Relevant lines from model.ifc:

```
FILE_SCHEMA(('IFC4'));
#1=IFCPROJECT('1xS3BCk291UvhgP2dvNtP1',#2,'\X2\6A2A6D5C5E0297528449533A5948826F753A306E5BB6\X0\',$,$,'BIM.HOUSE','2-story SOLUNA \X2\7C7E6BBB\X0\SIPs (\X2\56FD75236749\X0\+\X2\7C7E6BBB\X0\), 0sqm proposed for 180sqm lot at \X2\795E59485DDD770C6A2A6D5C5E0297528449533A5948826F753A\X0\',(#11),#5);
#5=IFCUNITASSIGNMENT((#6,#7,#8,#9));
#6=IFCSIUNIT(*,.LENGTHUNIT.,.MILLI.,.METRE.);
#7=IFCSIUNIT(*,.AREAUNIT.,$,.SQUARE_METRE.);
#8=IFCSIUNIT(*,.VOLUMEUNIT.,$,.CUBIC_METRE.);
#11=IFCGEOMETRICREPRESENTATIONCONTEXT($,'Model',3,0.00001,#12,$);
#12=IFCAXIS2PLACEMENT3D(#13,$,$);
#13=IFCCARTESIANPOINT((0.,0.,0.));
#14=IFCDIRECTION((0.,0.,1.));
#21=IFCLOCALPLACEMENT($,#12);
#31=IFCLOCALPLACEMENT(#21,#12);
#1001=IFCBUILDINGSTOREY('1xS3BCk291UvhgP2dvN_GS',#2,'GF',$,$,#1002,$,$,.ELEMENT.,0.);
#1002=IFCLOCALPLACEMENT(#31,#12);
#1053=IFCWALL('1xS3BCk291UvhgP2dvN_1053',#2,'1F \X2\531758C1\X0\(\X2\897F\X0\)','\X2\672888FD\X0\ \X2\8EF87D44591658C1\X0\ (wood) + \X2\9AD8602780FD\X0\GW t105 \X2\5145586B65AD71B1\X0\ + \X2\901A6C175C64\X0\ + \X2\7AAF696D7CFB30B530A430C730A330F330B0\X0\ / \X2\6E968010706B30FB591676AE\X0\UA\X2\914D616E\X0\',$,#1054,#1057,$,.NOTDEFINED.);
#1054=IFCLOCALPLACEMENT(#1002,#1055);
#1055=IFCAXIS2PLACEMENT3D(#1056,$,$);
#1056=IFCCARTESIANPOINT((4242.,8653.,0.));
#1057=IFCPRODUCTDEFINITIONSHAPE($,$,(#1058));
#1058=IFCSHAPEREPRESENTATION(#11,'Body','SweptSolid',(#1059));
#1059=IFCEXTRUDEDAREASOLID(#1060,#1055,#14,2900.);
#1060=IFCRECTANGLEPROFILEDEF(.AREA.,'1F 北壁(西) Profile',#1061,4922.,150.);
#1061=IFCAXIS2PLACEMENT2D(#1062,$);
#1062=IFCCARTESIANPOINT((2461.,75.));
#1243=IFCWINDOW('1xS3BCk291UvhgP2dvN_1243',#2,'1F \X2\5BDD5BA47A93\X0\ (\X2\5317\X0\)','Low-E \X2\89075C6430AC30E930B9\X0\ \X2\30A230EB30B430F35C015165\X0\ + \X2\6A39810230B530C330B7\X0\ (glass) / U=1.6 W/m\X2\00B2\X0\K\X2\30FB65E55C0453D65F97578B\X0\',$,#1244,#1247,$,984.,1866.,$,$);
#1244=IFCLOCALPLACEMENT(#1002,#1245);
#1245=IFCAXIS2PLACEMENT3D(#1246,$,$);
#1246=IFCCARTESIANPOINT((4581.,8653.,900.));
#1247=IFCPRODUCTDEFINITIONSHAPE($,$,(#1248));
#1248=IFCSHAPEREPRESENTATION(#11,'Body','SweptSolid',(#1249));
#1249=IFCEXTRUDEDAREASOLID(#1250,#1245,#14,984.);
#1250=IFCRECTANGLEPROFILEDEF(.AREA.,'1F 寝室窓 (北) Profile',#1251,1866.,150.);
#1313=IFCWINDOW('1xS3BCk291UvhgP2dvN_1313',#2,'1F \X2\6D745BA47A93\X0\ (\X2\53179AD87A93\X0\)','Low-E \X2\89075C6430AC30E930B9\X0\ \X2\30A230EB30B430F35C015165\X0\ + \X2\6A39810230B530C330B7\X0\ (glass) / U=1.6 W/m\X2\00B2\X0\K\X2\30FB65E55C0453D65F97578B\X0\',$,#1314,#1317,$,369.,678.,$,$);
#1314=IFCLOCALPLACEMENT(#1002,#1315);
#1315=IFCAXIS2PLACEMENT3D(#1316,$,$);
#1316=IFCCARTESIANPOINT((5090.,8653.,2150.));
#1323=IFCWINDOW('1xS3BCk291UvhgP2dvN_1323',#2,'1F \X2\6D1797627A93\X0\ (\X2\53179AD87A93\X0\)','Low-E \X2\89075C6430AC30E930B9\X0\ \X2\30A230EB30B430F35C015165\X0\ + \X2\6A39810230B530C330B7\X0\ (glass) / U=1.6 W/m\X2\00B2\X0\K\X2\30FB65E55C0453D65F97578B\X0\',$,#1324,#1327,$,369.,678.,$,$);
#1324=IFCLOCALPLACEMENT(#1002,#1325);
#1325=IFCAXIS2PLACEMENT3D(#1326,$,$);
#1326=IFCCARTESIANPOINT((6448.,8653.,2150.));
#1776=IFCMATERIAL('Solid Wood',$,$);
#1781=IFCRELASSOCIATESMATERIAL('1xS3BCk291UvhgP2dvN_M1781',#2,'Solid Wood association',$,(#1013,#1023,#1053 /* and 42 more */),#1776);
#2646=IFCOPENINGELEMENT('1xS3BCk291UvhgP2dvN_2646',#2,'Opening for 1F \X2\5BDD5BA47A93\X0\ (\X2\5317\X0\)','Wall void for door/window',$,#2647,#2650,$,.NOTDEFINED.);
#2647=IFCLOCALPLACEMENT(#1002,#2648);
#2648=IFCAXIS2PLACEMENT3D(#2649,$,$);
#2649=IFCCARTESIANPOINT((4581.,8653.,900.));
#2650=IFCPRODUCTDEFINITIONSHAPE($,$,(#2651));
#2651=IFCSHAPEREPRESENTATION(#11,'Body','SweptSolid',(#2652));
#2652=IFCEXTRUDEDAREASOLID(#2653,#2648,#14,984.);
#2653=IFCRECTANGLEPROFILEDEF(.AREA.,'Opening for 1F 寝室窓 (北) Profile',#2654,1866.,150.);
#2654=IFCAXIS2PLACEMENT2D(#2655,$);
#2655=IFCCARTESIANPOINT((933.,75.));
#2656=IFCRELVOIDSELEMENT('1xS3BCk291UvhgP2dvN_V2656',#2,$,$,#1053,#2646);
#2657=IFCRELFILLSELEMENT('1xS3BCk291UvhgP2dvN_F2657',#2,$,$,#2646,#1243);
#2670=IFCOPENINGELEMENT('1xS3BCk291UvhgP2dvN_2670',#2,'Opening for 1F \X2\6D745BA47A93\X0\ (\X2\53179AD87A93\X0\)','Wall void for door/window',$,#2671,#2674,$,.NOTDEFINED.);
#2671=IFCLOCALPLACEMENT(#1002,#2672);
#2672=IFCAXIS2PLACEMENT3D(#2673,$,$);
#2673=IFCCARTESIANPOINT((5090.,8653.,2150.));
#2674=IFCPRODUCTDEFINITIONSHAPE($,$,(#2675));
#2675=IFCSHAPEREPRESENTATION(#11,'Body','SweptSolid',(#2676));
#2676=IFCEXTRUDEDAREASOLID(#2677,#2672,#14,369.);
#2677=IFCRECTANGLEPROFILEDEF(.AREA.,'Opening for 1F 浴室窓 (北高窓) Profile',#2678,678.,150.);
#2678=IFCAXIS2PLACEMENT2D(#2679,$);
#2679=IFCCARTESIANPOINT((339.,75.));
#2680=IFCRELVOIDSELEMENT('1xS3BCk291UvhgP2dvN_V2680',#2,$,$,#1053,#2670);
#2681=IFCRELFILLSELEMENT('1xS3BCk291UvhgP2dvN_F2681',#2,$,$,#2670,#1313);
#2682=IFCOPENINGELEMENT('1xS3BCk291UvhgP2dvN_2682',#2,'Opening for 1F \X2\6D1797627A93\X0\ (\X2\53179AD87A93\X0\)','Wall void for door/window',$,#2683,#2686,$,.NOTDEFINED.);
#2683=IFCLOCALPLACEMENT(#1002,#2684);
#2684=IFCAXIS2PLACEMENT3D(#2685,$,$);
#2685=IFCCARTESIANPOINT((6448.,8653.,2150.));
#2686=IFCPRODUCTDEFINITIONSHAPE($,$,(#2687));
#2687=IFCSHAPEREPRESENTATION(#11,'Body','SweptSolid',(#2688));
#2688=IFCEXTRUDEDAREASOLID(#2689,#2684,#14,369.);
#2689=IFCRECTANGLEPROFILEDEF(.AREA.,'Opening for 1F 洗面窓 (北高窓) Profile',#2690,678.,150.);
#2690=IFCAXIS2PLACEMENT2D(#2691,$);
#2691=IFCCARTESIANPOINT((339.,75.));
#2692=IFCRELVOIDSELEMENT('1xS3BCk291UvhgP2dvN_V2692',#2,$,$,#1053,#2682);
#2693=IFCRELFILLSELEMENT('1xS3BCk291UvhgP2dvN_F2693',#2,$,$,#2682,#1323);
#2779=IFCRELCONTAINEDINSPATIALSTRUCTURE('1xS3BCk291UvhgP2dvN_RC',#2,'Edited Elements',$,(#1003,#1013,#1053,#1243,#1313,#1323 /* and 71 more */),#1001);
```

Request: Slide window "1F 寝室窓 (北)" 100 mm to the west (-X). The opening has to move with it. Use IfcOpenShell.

```python
import ifcopenshell
import ifcopenshell.api.geometry
import ifcopenshell.util.placement
import ifcopenshell.util.unit

model = ifcopenshell.open("model.ifc")
unit_scale = ifcopenshell.util.unit.calculate_unit_scale(model)

window = model.by_guid("1xS3BCk291UvhgP2dvN_1243")
opening = window.FillsVoids[0].RelatingOpeningElement
wall = opening.VoidsElements[0].RelatingBuildingElement

wall_matrix = ifcopenshell.util.placement.get_local_placement(wall.ObjectPlacement)
shift = wall_matrix[:3, 0] * -0.1 / unit_scale
before = ifcopenshell.util.placement.get_local_placement(window.ObjectPlacement)[:3, 3].copy()

# The window is not placed relative to its opening, so move both.
for product in (opening, window):
    matrix = ifcopenshell.util.placement.get_local_placement(product.ObjectPlacement)
    matrix[:3, 3] += shift
    ifcopenshell.api.geometry.edit_object_placement(model, product=product, matrix=matrix, is_si=False)

after = ifcopenshell.util.placement.get_local_placement(window.ObjectPlacement)[:3, 3]
print("window moved by", (after - before).round(3) + 0.0)

model.write("model_rev.ifc")
```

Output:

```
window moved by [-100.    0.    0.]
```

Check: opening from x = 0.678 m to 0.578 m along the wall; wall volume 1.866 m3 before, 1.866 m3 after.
